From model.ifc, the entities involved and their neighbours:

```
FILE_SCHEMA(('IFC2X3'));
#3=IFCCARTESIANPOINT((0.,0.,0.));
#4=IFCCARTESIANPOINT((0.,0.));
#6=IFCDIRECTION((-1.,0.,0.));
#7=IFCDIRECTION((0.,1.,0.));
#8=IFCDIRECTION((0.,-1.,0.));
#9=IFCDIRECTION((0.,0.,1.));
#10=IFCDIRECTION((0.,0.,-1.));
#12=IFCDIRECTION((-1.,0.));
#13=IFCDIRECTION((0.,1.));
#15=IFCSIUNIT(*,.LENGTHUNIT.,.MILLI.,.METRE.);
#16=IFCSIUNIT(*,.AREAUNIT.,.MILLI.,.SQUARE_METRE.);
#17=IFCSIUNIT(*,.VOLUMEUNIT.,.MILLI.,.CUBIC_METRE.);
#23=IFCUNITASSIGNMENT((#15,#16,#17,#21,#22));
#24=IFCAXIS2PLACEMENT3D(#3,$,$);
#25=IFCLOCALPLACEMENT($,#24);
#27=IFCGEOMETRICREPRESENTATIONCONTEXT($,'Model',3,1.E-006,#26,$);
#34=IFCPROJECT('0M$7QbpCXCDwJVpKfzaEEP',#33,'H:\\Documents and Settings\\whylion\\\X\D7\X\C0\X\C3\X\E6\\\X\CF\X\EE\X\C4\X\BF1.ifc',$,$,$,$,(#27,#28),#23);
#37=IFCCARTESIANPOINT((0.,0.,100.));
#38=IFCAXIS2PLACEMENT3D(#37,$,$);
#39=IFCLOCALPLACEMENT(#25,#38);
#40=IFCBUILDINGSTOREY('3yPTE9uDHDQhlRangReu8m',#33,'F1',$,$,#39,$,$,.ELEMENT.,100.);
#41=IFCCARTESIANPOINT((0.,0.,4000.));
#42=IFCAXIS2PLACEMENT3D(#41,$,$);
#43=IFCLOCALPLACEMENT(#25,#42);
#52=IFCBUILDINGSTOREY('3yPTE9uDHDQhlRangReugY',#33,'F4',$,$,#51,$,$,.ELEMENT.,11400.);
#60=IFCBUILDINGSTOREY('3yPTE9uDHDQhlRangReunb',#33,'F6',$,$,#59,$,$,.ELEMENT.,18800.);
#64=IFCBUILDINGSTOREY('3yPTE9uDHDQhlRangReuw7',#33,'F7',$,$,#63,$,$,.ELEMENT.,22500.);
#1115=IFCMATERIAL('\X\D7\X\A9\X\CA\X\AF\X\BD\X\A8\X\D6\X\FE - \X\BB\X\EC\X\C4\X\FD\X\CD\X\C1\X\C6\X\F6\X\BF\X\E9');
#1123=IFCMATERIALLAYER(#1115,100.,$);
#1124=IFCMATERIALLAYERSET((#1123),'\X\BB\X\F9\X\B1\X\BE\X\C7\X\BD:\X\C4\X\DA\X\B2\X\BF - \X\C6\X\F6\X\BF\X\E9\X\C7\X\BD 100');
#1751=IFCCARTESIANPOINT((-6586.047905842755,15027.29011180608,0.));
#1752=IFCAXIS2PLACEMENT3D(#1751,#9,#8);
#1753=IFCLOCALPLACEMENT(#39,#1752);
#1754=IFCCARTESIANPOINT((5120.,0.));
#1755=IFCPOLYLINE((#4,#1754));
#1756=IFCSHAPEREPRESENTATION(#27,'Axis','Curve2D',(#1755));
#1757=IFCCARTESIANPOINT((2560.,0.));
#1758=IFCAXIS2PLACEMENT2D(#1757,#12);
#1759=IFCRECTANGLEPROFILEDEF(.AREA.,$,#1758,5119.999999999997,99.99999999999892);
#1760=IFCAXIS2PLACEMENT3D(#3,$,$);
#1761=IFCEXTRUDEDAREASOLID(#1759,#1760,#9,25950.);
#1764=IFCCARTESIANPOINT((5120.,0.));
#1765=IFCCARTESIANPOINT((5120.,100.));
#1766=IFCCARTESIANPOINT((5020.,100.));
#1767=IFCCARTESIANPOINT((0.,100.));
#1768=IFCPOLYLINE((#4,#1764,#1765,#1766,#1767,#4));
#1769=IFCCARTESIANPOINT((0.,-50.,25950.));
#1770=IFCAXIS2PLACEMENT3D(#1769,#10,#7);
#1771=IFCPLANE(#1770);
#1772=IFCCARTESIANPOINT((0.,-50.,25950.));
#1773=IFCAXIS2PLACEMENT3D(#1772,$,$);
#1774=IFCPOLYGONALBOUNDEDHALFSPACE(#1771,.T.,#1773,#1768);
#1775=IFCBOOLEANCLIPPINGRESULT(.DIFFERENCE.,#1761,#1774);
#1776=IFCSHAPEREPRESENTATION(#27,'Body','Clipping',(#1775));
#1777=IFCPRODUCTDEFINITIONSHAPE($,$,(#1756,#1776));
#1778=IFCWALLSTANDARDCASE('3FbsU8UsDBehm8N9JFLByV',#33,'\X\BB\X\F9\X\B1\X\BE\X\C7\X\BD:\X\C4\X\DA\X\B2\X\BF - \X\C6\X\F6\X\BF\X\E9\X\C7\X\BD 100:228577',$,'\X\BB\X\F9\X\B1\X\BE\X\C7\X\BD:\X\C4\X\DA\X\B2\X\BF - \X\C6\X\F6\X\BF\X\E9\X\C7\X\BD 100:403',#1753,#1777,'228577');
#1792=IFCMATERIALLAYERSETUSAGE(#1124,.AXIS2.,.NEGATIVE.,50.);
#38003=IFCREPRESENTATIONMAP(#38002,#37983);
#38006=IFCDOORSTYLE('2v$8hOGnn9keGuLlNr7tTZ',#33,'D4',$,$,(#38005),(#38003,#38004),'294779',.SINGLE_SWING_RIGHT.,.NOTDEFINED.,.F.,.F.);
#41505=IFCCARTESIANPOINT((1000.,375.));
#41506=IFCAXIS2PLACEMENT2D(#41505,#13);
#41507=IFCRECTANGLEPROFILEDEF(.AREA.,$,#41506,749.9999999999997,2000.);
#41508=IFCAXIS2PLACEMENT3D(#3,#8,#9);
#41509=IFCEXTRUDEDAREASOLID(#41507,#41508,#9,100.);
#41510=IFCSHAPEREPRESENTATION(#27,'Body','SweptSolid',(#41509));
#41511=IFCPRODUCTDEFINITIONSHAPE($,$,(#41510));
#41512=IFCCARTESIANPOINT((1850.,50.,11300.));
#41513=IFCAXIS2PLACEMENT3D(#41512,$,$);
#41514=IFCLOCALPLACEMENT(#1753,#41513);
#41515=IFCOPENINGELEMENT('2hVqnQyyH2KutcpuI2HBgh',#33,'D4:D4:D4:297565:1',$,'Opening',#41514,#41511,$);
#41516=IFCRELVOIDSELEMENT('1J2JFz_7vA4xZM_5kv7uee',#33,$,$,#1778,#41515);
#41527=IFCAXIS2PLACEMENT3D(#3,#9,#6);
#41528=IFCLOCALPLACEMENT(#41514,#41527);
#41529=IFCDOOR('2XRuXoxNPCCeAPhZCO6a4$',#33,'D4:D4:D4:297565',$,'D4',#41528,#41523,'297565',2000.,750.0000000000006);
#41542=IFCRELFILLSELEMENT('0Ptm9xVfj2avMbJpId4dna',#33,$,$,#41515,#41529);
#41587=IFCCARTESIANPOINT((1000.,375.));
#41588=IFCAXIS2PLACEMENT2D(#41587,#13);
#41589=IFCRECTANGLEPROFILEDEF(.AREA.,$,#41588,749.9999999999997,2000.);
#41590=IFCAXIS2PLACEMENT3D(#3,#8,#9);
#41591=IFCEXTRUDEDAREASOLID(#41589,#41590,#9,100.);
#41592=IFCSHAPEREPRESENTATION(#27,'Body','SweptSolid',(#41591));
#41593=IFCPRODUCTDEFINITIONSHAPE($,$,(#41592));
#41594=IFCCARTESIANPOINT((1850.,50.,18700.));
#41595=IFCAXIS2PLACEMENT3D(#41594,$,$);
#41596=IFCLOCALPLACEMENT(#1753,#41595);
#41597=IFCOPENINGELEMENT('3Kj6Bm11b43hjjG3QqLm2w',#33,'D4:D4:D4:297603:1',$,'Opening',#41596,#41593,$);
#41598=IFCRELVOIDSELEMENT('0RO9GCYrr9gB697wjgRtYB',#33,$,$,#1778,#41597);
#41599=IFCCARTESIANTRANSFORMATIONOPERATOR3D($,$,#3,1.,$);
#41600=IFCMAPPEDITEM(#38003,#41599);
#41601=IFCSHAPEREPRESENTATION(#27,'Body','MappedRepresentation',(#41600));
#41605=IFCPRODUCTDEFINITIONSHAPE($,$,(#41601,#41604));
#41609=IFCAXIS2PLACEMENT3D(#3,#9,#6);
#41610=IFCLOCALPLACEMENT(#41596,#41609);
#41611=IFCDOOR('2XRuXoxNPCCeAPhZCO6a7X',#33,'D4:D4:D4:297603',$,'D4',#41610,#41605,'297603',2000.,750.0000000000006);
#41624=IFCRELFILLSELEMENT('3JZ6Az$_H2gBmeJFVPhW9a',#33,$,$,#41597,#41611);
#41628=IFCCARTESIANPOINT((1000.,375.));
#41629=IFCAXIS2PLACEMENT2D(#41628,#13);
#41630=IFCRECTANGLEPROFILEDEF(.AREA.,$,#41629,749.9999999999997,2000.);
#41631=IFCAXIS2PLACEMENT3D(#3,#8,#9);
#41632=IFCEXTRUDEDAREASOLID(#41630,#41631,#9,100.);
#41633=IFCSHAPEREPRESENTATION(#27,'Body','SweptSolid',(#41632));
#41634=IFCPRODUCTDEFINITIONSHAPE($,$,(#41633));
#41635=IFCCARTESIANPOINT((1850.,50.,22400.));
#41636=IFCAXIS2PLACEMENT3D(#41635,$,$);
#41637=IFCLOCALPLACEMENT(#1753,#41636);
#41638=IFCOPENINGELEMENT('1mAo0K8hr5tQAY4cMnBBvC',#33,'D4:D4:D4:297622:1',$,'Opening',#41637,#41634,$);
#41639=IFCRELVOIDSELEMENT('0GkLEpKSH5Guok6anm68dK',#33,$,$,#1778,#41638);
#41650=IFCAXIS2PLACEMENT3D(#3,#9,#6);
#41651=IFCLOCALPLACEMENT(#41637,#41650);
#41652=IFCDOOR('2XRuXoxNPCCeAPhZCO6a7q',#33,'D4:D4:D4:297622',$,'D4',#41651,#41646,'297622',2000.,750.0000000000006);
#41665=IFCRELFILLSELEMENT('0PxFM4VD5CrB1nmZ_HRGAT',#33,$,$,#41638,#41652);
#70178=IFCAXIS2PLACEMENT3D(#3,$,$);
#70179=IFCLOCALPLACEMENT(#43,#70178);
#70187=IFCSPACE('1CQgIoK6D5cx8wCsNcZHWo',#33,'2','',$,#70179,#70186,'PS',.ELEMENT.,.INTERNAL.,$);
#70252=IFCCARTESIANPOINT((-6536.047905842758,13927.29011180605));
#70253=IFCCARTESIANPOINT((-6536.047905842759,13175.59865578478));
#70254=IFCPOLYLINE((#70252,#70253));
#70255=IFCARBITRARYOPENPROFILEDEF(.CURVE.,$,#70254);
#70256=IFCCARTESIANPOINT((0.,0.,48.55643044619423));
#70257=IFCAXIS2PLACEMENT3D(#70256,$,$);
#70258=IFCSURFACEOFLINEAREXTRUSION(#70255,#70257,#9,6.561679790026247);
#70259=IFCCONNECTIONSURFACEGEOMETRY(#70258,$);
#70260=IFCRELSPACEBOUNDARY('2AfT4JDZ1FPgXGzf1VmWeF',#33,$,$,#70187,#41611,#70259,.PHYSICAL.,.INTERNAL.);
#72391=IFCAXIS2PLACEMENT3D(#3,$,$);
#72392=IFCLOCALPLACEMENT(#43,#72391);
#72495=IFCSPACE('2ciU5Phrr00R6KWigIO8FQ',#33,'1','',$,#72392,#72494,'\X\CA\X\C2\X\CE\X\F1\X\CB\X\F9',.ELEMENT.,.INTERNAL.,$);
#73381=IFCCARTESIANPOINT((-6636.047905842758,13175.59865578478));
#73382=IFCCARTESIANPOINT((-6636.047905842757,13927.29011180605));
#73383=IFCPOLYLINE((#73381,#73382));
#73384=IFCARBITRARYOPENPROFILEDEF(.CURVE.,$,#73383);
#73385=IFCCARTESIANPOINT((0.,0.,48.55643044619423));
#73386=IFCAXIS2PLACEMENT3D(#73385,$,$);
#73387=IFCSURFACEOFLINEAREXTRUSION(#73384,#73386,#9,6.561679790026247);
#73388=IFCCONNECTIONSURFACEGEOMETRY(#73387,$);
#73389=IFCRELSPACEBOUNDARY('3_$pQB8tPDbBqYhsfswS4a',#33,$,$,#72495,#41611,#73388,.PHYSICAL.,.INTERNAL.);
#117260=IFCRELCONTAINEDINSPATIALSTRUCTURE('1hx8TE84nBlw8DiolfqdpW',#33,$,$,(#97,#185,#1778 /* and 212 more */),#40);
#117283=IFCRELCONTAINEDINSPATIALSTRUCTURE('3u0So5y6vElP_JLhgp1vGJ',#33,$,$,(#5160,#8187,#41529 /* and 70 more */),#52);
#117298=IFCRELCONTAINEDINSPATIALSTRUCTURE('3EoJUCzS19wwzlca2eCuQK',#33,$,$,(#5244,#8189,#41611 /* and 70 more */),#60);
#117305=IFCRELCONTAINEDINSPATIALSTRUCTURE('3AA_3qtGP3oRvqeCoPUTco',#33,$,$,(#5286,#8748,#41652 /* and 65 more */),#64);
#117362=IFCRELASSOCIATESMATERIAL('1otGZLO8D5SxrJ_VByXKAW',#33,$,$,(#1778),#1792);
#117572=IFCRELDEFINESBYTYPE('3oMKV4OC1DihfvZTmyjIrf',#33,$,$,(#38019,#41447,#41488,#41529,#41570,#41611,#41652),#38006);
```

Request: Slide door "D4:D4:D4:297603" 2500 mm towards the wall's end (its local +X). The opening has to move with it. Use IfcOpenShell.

```python
import numpy as np
import ifcopenshell
import ifcopenshell.api.geometry
import ifcopenshell.util.placement
import ifcopenshell.util.unit

model = ifcopenshell.open("model.ifc")
unit_scale = ifcopenshell.util.unit.calculate_unit_scale(model)

door = model.by_guid("2XRuXoxNPCCeAPhZCO6a7X")
opening = door.FillsVoids[0].RelatingOpeningElement
wall = opening.VoidsElements[0].RelatingBuildingElement

wall_matrix = ifcopenshell.util.placement.get_local_placement(wall.ObjectPlacement)
shift = wall_matrix[:3, 0] * 2.5 / unit_scale
before = ifcopenshell.util.placement.get_local_placement(door.ObjectPlacement)[:3, 3].copy()

# The door is placed relative to its opening, so it follows when the opening moves.
matrix = ifcopenshell.util.placement.get_local_placement(opening.ObjectPlacement)
matrix[:3, 3] += shift
ifcopenshell.api.geometry.edit_object_placement(
    model, product=opening, matrix=matrix, is_si=False, should_transform_children=True
)

# Space boundary surfaces are stored in each space's coordinates; move them too.
for rel in door.ProvidesBoundaries:
    if not rel.ConnectionGeometry:
        continue
    surface = rel.ConnectionGeometry.SurfaceOnRelatingElement
    space_matrix = ifcopenshell.util.placement.get_local_placement(rel.RelatingSpace.ObjectPlacement)
    point = np.array(surface.Position.Location.Coordinates) + space_matrix[:3, :3].T @ shift
    surface.Position = model.createIfcAxis2Placement3D(
        model.createIfcCartesianPoint(point.tolist()), surface.Position.Axis, surface.Position.RefDirection
    )

after = ifcopenshell.util.placement.get_local_placement(door.ObjectPlacement)[:3, 3]
print("door moved by", (after - before).round(3) + 0.0)

model.write("model_edited.ifc")
```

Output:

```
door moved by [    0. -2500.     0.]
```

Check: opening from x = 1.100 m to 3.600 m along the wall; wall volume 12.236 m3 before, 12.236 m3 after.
